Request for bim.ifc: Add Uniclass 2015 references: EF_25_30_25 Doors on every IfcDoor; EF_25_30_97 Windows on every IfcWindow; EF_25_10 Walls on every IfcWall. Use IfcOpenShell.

First a look at what the model holds.

```python
import ifcopenshell

model = ifcopenshell.open("bim.ifc")
print(model.schema)
print("classifications:", [c.Name for c in model.by_type("IfcClassification")])
for ifc_class in ("IfcDoor", "IfcRoof", "IfcStair", "IfcWall", "IfcWindow"):
    print(ifc_class, len(model.by_type(ifc_class)))
```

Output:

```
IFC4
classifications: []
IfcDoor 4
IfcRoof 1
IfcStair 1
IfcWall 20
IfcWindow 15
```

```python
import ifcopenshell
import ifcopenshell.api.classification

model = ifcopenshell.open("bim.ifc")

system = ifcopenshell.api.classification.add_classification(model, classification="Uniclass 2015")

codes = {
    "IfcDoor": ("EF_25_30_25", "Doors"),
    "IfcWindow": ("EF_25_30_97", "Windows"),
    "IfcWall": ("EF_25_10", "Walls"),
}
for ifc_class, (code, name) in codes.items():
    products = model.by_type(ifc_class)
    ifcopenshell.api.classification.add_reference(
        model, products=products, classification=system, identification=code, name=name
    )
    print(code, len(products))

model.write("bim_rev.ifc")
```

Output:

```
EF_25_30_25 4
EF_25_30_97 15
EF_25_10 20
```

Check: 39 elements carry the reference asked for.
